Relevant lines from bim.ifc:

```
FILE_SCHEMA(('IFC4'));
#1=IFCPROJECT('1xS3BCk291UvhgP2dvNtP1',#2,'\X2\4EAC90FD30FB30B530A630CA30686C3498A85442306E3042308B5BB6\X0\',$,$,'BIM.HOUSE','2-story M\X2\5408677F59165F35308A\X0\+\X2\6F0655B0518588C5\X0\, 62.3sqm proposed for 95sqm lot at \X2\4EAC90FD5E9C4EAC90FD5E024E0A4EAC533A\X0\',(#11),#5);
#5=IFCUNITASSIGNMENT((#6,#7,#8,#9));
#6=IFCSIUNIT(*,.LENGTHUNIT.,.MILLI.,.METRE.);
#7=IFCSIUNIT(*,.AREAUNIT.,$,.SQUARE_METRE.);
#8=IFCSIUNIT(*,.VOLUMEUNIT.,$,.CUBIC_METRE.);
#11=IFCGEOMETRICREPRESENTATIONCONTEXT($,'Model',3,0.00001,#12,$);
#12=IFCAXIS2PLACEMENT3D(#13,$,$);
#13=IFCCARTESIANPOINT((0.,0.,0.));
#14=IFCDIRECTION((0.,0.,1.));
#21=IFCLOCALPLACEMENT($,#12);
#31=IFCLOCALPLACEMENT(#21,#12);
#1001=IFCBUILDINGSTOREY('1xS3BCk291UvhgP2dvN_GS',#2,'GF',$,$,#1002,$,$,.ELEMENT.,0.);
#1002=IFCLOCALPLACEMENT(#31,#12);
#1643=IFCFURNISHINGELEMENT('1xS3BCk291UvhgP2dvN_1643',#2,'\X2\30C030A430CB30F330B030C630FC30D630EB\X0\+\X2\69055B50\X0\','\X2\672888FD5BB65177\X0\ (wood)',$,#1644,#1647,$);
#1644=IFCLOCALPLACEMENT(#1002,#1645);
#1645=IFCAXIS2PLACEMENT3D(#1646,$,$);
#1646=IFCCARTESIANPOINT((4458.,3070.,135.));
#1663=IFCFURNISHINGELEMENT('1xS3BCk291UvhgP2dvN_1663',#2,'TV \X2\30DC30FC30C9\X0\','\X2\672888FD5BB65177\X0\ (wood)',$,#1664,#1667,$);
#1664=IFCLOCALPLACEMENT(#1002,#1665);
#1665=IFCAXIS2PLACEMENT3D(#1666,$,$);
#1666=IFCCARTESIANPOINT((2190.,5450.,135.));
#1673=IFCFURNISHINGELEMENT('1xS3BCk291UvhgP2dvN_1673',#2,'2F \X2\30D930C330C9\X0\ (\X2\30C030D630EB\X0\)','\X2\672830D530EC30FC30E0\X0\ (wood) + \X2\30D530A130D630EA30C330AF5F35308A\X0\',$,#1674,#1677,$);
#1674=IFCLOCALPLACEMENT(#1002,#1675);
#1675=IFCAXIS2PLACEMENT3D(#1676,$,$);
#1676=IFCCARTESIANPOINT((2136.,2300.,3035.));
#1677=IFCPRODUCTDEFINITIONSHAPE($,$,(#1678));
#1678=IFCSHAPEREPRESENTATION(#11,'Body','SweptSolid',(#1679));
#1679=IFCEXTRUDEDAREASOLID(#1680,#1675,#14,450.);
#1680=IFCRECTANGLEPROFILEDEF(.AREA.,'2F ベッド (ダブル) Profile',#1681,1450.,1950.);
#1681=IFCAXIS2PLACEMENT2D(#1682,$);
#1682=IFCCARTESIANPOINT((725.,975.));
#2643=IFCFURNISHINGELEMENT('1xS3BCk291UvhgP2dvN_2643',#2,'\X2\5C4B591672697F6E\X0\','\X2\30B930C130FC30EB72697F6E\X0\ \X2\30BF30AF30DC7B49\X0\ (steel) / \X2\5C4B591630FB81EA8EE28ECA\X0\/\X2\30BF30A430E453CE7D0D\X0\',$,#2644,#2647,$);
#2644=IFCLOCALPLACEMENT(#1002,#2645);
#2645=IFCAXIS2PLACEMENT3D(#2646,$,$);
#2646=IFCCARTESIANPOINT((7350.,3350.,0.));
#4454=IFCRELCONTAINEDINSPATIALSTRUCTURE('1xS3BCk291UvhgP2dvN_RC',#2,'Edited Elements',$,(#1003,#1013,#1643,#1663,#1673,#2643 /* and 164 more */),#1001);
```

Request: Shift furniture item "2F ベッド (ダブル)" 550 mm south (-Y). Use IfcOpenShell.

```python
import ifcopenshell
import ifcopenshell.api.geometry
import ifcopenshell.util.placement
import ifcopenshell.util.unit

model = ifcopenshell.open("bim.ifc")
unit_scale = ifcopenshell.util.unit.calculate_unit_scale(model)

item = model.by_guid("1xS3BCk291UvhgP2dvN_1673")
matrix = ifcopenshell.util.placement.get_local_placement(item.ObjectPlacement)
matrix[1, 3] -= 0.55 / unit_scale
ifcopenshell.api.geometry.edit_object_placement(model, product=item, matrix=matrix, is_si=False)

print(ifcopenshell.util.placement.get_local_placement(item.ObjectPlacement).round(3) + 0.0)

model.write("bim-out.ifc")
```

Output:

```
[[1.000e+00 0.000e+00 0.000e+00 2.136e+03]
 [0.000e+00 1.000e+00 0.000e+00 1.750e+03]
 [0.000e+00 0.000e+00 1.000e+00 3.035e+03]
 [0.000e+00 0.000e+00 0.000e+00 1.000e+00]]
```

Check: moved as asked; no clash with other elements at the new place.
